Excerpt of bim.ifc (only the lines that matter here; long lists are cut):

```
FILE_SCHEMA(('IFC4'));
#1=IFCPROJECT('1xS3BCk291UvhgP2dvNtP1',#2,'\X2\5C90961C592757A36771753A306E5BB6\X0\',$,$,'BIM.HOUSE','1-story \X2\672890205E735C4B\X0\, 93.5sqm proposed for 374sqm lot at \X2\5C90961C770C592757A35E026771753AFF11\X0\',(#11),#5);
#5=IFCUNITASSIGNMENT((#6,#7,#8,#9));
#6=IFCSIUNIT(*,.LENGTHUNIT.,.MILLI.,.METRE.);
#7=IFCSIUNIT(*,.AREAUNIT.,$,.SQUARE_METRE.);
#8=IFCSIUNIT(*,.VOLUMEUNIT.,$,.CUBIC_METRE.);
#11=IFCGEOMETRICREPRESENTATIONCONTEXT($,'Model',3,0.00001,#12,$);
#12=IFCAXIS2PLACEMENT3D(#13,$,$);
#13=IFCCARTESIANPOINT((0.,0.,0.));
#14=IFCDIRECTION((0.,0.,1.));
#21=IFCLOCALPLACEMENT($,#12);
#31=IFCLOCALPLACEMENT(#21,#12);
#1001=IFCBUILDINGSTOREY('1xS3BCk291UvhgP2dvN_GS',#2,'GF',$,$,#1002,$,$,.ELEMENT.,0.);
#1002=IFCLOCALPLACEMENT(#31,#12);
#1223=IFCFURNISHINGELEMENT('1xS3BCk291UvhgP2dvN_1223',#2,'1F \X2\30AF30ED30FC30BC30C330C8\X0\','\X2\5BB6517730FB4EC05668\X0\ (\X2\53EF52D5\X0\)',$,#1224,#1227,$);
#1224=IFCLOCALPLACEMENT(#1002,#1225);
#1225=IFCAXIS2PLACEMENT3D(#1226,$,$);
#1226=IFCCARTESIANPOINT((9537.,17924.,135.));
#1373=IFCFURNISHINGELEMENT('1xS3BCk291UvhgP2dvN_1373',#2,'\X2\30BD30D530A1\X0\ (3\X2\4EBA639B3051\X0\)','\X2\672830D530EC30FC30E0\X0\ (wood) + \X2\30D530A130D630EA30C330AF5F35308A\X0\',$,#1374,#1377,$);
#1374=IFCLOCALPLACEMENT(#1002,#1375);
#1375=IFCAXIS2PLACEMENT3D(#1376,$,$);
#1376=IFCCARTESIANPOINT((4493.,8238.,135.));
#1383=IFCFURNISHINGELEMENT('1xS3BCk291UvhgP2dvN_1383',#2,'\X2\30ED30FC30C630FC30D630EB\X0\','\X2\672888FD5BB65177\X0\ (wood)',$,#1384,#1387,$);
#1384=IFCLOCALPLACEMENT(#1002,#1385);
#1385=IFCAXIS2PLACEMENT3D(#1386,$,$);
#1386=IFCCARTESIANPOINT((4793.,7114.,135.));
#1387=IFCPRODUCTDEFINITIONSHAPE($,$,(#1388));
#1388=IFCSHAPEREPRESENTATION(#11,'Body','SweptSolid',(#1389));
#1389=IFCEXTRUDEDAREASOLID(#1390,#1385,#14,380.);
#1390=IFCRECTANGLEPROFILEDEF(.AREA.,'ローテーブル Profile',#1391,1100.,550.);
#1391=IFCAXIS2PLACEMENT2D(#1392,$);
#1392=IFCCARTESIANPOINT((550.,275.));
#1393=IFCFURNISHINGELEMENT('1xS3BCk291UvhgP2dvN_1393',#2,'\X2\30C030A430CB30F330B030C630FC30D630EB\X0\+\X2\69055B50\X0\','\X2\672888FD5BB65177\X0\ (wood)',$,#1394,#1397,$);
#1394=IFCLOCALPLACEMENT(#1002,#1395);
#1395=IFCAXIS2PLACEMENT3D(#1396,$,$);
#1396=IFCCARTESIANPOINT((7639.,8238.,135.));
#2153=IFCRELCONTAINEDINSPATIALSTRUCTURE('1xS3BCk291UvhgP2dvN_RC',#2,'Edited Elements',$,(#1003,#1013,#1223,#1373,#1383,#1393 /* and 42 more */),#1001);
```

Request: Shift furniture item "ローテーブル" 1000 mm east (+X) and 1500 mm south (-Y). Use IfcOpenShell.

```python
import ifcopenshell
import ifcopenshell.api.geometry
import ifcopenshell.util.placement
import ifcopenshell.util.unit

model = ifcopenshell.open("bim.ifc")
unit_scale = ifcopenshell.util.unit.calculate_unit_scale(model)

item = model.by_id(1383)
matrix = ifcopenshell.util.placement.get_local_placement(item.ObjectPlacement)
matrix[0, 3] += 1 / unit_scale
matrix[1, 3] -= 1.5 / unit_scale
ifcopenshell.api.geometry.edit_object_placement(model, product=item, matrix=matrix, is_si=False)

print(ifcopenshell.util.placement.get_local_placement(item.ObjectPlacement).round(3) + 0.0)

model.write("bim-out.ifc")
```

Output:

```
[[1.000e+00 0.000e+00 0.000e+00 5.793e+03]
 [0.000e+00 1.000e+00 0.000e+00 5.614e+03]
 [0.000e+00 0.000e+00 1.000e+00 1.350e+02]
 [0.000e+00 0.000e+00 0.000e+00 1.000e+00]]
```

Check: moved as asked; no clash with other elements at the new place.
